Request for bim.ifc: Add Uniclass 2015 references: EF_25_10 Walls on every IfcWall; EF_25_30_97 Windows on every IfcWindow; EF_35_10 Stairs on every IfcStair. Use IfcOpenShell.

First a look at what the model holds.

```python
import ifcopenshell

model = ifcopenshell.open("bim.ifc")
print(model.schema)
print("classifications:", [c.Name for c in model.by_type("IfcClassification")])
for ifc_class in ("IfcDoor", "IfcRoof", "IfcStair", "IfcWall", "IfcWindow"):
    print(ifc_class, len(model.by_type(ifc_class)))
```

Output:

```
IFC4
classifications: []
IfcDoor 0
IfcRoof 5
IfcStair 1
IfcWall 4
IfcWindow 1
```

```python
import ifcopenshell
import ifcopenshell.api.classification

model = ifcopenshell.open("bim.ifc")

system = ifcopenshell.api.classification.add_classification(model, classification="Uniclass 2015")

codes = {
    "IfcWall": ("EF_25_10", "Walls"),
    "IfcWindow": ("EF_25_30_97", "Windows"),
    "IfcStair": ("EF_35_10", "Stairs"),
}
for ifc_class, (code, name) in codes.items():
    products = model.by_type(ifc_class)
    ifcopenshell.api.classification.add_reference(
        model, products=products, classification=system, identification=code, name=name
    )
    print(code, len(products))

model.write("bim_edited.ifc")
```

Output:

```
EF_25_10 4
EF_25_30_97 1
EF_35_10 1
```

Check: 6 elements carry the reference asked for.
